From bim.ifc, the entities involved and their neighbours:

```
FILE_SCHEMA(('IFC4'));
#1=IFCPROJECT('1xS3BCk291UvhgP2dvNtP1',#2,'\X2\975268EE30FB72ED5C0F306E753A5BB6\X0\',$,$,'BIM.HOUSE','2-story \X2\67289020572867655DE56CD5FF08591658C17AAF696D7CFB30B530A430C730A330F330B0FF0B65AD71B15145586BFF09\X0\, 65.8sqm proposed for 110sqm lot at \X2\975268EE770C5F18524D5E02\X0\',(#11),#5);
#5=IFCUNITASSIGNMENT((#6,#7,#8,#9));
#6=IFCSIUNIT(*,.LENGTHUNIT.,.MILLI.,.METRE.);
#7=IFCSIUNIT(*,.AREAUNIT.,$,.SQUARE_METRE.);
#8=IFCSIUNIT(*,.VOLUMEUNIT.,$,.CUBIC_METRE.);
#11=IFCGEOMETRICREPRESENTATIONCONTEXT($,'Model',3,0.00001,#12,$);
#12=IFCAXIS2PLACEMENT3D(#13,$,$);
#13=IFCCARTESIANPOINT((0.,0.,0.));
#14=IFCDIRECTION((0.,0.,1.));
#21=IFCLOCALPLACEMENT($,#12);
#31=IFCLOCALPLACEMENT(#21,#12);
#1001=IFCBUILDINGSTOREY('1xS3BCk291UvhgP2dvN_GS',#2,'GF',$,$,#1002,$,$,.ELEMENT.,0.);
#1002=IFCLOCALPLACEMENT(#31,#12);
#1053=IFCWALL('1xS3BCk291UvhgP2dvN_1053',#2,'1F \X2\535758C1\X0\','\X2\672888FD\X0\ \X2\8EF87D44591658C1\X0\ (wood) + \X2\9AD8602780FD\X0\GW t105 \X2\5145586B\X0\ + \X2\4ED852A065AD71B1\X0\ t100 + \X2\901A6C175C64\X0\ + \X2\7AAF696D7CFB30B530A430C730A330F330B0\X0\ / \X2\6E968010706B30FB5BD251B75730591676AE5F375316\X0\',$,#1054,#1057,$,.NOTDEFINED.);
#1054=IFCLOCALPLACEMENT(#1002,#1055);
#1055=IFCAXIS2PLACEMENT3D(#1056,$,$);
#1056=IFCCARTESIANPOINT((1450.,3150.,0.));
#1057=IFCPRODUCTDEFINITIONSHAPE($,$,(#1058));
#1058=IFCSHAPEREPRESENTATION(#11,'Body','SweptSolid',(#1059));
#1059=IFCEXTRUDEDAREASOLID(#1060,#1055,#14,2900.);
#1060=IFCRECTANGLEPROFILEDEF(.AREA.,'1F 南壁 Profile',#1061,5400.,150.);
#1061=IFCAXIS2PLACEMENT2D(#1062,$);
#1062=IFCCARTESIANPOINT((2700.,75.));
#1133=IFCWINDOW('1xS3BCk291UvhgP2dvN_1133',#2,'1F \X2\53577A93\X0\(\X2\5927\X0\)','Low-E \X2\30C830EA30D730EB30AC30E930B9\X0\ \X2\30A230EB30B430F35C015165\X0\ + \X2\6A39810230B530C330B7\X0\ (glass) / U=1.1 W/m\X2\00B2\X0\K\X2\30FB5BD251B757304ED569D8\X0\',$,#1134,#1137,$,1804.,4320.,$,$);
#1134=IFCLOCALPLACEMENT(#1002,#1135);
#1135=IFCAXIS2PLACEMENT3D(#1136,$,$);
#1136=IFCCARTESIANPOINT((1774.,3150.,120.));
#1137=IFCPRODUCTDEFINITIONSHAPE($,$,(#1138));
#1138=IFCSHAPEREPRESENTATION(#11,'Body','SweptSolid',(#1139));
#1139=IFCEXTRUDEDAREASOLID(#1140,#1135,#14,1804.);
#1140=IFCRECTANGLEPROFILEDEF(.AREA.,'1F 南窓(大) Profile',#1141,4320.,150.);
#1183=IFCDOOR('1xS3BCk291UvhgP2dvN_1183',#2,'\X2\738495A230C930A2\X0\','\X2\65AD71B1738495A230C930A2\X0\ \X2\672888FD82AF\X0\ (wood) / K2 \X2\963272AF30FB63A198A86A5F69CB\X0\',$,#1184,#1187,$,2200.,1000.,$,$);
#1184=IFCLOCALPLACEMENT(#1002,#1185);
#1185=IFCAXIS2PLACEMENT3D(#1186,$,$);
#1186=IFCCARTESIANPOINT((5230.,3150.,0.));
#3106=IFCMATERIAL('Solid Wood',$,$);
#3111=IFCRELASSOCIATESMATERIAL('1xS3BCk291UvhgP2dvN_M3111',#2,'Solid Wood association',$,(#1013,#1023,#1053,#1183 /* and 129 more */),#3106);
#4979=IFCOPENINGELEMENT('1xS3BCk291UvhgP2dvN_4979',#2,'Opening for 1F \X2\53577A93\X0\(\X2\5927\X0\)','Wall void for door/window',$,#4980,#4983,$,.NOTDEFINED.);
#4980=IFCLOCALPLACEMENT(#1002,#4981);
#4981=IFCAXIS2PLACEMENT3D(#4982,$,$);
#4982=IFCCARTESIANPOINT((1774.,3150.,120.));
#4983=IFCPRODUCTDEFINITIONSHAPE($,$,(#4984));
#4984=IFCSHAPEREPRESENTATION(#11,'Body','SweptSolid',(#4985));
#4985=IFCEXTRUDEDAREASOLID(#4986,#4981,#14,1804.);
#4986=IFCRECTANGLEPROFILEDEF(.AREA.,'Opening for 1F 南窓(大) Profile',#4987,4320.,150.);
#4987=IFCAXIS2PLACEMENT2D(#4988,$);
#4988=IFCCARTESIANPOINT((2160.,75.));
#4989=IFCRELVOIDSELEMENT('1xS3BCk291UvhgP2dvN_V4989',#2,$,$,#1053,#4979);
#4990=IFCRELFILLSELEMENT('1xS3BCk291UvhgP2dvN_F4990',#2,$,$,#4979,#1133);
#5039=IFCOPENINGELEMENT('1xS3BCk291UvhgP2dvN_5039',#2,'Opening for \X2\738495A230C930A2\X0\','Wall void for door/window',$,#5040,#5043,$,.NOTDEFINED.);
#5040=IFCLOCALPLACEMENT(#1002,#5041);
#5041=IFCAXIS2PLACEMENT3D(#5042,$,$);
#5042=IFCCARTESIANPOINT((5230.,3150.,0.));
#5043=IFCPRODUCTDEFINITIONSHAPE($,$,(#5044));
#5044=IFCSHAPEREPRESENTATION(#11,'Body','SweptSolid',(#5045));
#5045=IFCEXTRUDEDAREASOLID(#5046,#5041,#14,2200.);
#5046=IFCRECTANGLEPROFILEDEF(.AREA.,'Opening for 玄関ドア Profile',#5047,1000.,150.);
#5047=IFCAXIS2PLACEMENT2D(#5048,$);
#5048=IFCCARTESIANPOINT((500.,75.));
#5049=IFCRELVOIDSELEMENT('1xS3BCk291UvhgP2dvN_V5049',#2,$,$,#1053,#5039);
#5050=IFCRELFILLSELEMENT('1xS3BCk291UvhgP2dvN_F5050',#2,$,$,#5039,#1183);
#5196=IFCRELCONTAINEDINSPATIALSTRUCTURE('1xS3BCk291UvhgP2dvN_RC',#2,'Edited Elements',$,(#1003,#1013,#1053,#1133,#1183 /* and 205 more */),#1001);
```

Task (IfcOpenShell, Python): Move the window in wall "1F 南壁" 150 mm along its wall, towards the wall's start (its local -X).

```python
import ifcopenshell
import ifcopenshell.api.geometry
import ifcopenshell.util.placement

model = ifcopenshell.open("bim.ifc")

window = model.by_guid("1xS3BCk291UvhgP2dvN_1133")
opening = window.FillsVoids[0].RelatingOpeningElement
wall = opening.VoidsElements[0].RelatingBuildingElement

wall_matrix = ifcopenshell.util.placement.get_local_placement(wall.ObjectPlacement)
shift = wall_matrix[:3, 0] * -150.0
before = ifcopenshell.util.placement.get_local_placement(window.ObjectPlacement)[:3, 3].copy()

# The window is not placed relative to its opening, so move both.
for product in (opening, window):
    matrix = ifcopenshell.util.placement.get_local_placement(product.ObjectPlacement)
    matrix[:3, 3] += shift
    ifcopenshell.api.geometry.edit_object_placement(model, product=product, matrix=matrix, is_si=False)

after = ifcopenshell.util.placement.get_local_placement(window.ObjectPlacement)[:3, 3]
print("window moved by", (after - before).round(3) + 0.0)

model.write("bim_edited.ifc")
```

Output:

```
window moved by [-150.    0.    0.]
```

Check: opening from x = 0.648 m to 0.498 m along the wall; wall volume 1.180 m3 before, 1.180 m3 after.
